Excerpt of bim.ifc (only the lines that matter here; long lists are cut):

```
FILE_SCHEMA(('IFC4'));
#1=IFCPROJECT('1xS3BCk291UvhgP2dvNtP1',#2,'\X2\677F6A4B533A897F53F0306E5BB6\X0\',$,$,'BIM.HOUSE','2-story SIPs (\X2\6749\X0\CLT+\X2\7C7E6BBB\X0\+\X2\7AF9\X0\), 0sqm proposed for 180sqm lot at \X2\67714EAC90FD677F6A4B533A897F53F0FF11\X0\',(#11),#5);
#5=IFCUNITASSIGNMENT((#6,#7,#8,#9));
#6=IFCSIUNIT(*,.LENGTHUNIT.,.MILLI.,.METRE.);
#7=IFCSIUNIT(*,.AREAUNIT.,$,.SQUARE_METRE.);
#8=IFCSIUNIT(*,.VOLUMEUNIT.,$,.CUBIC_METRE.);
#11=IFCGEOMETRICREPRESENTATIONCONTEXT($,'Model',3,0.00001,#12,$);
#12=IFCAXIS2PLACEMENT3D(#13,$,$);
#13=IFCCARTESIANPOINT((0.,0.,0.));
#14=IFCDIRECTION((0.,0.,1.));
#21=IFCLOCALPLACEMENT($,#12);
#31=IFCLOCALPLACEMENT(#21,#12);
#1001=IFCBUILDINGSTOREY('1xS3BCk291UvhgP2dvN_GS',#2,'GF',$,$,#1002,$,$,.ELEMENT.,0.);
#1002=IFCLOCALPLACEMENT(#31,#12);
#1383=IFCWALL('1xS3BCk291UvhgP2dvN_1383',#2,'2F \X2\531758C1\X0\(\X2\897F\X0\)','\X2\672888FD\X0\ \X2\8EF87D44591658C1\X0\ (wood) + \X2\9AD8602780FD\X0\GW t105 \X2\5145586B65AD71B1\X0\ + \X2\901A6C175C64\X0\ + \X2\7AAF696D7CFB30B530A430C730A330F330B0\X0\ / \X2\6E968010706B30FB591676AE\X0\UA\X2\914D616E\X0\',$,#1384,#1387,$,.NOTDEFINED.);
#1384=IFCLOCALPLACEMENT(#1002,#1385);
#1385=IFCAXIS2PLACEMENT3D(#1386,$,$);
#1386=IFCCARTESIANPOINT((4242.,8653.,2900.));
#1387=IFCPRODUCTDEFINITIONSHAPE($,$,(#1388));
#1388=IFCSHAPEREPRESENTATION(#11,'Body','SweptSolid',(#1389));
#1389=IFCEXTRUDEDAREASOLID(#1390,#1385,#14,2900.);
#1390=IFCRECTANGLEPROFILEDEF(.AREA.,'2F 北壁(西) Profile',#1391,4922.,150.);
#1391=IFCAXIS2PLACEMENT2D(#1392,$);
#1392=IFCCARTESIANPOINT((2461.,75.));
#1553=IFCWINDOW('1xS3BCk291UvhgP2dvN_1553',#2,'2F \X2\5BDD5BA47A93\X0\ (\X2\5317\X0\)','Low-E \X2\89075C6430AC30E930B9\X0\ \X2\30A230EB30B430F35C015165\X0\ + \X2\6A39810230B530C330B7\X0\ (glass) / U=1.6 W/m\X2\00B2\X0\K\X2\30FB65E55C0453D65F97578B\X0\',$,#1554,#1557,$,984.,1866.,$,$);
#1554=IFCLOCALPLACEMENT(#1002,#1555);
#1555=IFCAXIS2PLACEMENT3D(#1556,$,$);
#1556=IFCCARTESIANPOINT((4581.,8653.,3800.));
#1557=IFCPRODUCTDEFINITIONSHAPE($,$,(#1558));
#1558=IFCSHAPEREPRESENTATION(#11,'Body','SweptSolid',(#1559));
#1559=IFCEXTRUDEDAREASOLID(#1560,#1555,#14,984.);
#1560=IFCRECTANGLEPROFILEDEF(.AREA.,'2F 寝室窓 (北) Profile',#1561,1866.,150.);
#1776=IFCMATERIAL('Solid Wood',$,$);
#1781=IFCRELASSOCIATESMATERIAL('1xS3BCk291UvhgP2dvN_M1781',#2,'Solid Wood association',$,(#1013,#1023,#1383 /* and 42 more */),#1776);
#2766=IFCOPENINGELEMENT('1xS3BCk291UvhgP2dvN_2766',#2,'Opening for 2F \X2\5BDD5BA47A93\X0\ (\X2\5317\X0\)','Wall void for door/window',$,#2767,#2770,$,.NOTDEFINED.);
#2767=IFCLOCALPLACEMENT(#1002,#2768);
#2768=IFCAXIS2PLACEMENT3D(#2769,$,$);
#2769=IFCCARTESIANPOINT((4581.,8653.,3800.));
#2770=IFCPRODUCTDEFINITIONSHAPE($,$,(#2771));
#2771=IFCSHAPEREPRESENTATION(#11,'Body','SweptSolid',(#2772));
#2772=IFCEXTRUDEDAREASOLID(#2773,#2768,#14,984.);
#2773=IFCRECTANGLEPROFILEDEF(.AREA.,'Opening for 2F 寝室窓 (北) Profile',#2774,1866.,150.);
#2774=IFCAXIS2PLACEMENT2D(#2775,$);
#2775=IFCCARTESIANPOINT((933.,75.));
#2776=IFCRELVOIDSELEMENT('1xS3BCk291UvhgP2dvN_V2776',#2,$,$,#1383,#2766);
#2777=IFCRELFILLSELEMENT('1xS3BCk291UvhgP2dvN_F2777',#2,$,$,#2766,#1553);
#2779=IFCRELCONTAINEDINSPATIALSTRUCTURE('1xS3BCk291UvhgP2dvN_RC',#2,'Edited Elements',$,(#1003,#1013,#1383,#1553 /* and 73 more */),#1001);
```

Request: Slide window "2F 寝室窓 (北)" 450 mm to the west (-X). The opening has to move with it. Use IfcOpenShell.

```python
import ifcopenshell
import ifcopenshell.api.geometry
import ifcopenshell.util.placement
import ifcopenshell.util.unit

model = ifcopenshell.open("bim.ifc")
unit_scale = ifcopenshell.util.unit.calculate_unit_scale(model)

window = model.by_guid("1xS3BCk291UvhgP2dvN_1553")
opening = window.FillsVoids[0].RelatingOpeningElement
wall = opening.VoidsElements[0].RelatingBuildingElement

wall_matrix = ifcopenshell.util.placement.get_local_placement(wall.ObjectPlacement)
shift = wall_matrix[:3, 0] * -0.45 / unit_scale
before = ifcopenshell.util.placement.get_local_placement(window.ObjectPlacement)[:3, 3].copy()

# The window is not placed relative to its opening, so move both.
for product in (opening, window):
    matrix = ifcopenshell.util.placement.get_local_placement(product.ObjectPlacement)
    matrix[:3, 3] += shift
    ifcopenshell.api.geometry.edit_object_placement(model, product=product, matrix=matrix, is_si=False)

after = ifcopenshell.util.placement.get_local_placement(window.ObjectPlacement)[:3, 3]
print("window moved by", (after - before).round(3) + 0.0)

model.write("bim_edited.ifc")
```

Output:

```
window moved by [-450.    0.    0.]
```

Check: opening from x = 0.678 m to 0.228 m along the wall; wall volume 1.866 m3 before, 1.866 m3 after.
